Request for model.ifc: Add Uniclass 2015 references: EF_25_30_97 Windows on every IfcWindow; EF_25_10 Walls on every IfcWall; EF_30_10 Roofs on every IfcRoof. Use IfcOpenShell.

First a look at what the model holds.

```python
import ifcopenshell

model = ifcopenshell.open("model.ifc")
print(model.schema)
print("classifications:", [c.Name for c in model.by_type("IfcClassification")])
for ifc_class in ("IfcDoor", "IfcRoof", "IfcStair", "IfcWall", "IfcWindow"):
    print(ifc_class, len(model.by_type(ifc_class)))
```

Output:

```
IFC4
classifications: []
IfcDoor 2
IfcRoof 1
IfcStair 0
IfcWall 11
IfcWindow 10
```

```python
import ifcopenshell
import ifcopenshell.api.classification

model = ifcopenshell.open("model.ifc")

system = ifcopenshell.api.classification.add_classification(model, classification="Uniclass 2015")

codes = {
    "IfcWindow": ("EF_25_30_97", "Windows"),
    "IfcWall": ("EF_25_10", "Walls"),
    "IfcRoof": ("EF_30_10", "Roofs"),
}
for ifc_class, (code, name) in codes.items():
    products = model.by_type(ifc_class)
    ifcopenshell.api.classification.add_reference(
        model, products=products, classification=system, identification=code, name=name
    )
    print(code, len(products))

model.write("model_v2.ifc")
```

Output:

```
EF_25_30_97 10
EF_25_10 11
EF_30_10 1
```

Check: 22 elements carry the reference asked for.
